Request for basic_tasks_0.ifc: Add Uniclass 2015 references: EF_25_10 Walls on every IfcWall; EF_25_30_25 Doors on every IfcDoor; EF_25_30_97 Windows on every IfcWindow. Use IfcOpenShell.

First a look at what the model holds.

```python
import ifcopenshell

model = ifcopenshell.open("basic_tasks_0.ifc")
print(model.schema)
print("classifications:", [c.Name for c in model.by_type("IfcClassification")])
for ifc_class in ("IfcDoor", "IfcRoof", "IfcStair", "IfcWall", "IfcWindow"):
    print(ifc_class, len(model.by_type(ifc_class)))
```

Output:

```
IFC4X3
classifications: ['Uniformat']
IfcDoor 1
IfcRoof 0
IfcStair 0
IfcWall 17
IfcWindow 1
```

```python
import ifcopenshell
import ifcopenshell.api.classification

model = ifcopenshell.open("basic_tasks_0.ifc")

system = ifcopenshell.api.classification.add_classification(model, classification="Uniclass 2015")

codes = {
    "IfcWall": ("EF_25_10", "Walls"),
    "IfcDoor": ("EF_25_30_25", "Doors"),
    "IfcWindow": ("EF_25_30_97", "Windows"),
}
for ifc_class, (code, name) in codes.items():
    products = model.by_type(ifc_class)
    ifcopenshell.api.classification.add_reference(
        model, products=products, classification=system, identification=code, name=name
    )
    print(code, len(products))

model.write("basic_tasks_0_v2.ifc")
```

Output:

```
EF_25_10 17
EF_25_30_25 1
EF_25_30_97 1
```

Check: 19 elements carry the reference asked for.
